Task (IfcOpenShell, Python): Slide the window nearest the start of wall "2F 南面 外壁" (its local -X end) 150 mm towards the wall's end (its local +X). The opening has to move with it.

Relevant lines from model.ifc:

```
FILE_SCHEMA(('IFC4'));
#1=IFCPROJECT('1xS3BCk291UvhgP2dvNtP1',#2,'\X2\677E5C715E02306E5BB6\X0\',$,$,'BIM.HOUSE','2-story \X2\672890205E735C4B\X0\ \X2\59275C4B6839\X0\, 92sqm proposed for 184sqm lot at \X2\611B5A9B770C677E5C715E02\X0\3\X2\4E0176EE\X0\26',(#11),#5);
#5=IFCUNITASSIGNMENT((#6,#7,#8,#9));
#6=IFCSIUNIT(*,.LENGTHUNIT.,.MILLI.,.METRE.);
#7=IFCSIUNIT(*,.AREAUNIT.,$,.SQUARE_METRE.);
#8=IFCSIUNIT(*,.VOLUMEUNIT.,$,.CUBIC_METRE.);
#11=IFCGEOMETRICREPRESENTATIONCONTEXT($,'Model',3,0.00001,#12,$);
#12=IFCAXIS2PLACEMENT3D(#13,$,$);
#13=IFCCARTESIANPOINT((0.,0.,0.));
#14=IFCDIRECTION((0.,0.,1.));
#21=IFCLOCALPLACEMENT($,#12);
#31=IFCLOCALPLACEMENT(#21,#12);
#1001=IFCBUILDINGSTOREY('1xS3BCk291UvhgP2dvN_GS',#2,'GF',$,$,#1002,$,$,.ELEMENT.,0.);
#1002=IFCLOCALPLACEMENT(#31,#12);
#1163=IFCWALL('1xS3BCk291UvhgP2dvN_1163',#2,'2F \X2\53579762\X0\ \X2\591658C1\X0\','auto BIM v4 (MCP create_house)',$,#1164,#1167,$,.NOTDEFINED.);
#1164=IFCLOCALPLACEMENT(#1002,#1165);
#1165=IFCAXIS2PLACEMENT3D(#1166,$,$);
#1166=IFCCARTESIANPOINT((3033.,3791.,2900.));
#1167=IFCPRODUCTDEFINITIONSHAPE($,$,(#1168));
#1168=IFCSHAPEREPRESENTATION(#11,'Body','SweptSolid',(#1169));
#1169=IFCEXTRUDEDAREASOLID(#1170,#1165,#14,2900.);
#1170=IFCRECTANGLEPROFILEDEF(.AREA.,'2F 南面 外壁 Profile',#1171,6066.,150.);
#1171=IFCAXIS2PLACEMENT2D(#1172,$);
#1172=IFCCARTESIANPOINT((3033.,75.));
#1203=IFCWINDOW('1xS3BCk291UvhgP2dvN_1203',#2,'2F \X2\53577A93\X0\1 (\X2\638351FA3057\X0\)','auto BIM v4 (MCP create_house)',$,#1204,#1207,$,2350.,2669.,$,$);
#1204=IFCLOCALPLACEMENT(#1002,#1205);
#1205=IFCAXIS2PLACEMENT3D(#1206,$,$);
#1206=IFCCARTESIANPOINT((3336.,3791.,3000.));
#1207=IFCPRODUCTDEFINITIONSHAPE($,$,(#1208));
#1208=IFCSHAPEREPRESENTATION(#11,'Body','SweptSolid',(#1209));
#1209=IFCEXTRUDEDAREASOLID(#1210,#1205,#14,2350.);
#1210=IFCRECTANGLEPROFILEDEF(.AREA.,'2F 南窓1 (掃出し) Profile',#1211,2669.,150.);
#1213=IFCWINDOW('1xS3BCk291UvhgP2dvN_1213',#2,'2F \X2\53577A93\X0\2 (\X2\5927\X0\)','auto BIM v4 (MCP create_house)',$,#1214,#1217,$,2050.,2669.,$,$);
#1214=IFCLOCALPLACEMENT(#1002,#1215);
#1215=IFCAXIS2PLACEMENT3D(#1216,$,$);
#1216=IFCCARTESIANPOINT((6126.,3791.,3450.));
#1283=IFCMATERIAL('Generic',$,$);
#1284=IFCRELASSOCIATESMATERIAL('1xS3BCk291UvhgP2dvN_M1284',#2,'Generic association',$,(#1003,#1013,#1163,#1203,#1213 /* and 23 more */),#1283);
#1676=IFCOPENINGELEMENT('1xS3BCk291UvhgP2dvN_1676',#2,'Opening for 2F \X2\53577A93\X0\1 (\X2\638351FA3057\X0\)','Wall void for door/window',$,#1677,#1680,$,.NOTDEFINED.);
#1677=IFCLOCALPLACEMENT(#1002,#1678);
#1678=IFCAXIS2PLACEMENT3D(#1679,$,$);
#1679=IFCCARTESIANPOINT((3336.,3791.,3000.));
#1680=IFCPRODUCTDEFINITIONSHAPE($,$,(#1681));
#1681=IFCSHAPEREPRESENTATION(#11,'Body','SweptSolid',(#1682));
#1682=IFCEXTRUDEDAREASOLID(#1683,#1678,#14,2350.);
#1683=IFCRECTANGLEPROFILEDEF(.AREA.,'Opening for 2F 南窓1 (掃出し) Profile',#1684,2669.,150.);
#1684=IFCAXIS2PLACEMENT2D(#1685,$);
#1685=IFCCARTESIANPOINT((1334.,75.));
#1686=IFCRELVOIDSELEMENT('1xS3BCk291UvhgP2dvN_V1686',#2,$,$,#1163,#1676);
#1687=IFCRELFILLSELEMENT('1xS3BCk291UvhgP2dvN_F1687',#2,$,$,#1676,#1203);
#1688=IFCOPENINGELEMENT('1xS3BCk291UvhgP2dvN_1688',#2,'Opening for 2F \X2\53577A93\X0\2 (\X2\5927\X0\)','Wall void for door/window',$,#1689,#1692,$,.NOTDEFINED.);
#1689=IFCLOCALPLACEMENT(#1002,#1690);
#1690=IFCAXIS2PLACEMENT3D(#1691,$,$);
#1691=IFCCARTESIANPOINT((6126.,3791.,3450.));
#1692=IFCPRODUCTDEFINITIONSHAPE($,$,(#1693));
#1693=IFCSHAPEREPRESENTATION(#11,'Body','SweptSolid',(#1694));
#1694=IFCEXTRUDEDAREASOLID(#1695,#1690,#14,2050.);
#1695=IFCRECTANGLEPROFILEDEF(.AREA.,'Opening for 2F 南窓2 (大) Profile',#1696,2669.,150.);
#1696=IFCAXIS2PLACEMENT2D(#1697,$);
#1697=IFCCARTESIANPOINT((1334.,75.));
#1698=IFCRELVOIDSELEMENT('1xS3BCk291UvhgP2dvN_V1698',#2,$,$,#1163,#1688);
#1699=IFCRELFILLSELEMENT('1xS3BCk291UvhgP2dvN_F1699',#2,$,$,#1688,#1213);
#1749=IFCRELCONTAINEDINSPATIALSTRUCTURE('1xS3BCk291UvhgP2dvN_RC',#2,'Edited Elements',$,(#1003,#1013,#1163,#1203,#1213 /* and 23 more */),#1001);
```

```python
import ifcopenshell
import ifcopenshell.api.geometry
import ifcopenshell.util.placement
import ifcopenshell.util.unit

model = ifcopenshell.open("model.ifc")
unit_scale = ifcopenshell.util.unit.calculate_unit_scale(model)

window = model.by_guid("1xS3BCk291UvhgP2dvN_1203")
opening = window.FillsVoids[0].RelatingOpeningElement
wall = opening.VoidsElements[0].RelatingBuildingElement

wall_matrix = ifcopenshell.util.placement.get_local_placement(wall.ObjectPlacement)
shift = wall_matrix[:3, 0] * 0.15 / unit_scale
before = ifcopenshell.util.placement.get_local_placement(window.ObjectPlacement)[:3, 3].copy()

# The window is not placed relative to its opening, so move both.
for product in (opening, window):
    matrix = ifcopenshell.util.placement.get_local_placement(product.ObjectPlacement)
    matrix[:3, 3] += shift
    ifcopenshell.api.geometry.edit_object_placement(model, product=product, matrix=matrix, is_si=False)

after = ifcopenshell.util.placement.get_local_placement(window.ObjectPlacement)[:3, 3]
print("window moved by", (after - before).round(3) + 0.0)

model.write("model_rev.ifc")
```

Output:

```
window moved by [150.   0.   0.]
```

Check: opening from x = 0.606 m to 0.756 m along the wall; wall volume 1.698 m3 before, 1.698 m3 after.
